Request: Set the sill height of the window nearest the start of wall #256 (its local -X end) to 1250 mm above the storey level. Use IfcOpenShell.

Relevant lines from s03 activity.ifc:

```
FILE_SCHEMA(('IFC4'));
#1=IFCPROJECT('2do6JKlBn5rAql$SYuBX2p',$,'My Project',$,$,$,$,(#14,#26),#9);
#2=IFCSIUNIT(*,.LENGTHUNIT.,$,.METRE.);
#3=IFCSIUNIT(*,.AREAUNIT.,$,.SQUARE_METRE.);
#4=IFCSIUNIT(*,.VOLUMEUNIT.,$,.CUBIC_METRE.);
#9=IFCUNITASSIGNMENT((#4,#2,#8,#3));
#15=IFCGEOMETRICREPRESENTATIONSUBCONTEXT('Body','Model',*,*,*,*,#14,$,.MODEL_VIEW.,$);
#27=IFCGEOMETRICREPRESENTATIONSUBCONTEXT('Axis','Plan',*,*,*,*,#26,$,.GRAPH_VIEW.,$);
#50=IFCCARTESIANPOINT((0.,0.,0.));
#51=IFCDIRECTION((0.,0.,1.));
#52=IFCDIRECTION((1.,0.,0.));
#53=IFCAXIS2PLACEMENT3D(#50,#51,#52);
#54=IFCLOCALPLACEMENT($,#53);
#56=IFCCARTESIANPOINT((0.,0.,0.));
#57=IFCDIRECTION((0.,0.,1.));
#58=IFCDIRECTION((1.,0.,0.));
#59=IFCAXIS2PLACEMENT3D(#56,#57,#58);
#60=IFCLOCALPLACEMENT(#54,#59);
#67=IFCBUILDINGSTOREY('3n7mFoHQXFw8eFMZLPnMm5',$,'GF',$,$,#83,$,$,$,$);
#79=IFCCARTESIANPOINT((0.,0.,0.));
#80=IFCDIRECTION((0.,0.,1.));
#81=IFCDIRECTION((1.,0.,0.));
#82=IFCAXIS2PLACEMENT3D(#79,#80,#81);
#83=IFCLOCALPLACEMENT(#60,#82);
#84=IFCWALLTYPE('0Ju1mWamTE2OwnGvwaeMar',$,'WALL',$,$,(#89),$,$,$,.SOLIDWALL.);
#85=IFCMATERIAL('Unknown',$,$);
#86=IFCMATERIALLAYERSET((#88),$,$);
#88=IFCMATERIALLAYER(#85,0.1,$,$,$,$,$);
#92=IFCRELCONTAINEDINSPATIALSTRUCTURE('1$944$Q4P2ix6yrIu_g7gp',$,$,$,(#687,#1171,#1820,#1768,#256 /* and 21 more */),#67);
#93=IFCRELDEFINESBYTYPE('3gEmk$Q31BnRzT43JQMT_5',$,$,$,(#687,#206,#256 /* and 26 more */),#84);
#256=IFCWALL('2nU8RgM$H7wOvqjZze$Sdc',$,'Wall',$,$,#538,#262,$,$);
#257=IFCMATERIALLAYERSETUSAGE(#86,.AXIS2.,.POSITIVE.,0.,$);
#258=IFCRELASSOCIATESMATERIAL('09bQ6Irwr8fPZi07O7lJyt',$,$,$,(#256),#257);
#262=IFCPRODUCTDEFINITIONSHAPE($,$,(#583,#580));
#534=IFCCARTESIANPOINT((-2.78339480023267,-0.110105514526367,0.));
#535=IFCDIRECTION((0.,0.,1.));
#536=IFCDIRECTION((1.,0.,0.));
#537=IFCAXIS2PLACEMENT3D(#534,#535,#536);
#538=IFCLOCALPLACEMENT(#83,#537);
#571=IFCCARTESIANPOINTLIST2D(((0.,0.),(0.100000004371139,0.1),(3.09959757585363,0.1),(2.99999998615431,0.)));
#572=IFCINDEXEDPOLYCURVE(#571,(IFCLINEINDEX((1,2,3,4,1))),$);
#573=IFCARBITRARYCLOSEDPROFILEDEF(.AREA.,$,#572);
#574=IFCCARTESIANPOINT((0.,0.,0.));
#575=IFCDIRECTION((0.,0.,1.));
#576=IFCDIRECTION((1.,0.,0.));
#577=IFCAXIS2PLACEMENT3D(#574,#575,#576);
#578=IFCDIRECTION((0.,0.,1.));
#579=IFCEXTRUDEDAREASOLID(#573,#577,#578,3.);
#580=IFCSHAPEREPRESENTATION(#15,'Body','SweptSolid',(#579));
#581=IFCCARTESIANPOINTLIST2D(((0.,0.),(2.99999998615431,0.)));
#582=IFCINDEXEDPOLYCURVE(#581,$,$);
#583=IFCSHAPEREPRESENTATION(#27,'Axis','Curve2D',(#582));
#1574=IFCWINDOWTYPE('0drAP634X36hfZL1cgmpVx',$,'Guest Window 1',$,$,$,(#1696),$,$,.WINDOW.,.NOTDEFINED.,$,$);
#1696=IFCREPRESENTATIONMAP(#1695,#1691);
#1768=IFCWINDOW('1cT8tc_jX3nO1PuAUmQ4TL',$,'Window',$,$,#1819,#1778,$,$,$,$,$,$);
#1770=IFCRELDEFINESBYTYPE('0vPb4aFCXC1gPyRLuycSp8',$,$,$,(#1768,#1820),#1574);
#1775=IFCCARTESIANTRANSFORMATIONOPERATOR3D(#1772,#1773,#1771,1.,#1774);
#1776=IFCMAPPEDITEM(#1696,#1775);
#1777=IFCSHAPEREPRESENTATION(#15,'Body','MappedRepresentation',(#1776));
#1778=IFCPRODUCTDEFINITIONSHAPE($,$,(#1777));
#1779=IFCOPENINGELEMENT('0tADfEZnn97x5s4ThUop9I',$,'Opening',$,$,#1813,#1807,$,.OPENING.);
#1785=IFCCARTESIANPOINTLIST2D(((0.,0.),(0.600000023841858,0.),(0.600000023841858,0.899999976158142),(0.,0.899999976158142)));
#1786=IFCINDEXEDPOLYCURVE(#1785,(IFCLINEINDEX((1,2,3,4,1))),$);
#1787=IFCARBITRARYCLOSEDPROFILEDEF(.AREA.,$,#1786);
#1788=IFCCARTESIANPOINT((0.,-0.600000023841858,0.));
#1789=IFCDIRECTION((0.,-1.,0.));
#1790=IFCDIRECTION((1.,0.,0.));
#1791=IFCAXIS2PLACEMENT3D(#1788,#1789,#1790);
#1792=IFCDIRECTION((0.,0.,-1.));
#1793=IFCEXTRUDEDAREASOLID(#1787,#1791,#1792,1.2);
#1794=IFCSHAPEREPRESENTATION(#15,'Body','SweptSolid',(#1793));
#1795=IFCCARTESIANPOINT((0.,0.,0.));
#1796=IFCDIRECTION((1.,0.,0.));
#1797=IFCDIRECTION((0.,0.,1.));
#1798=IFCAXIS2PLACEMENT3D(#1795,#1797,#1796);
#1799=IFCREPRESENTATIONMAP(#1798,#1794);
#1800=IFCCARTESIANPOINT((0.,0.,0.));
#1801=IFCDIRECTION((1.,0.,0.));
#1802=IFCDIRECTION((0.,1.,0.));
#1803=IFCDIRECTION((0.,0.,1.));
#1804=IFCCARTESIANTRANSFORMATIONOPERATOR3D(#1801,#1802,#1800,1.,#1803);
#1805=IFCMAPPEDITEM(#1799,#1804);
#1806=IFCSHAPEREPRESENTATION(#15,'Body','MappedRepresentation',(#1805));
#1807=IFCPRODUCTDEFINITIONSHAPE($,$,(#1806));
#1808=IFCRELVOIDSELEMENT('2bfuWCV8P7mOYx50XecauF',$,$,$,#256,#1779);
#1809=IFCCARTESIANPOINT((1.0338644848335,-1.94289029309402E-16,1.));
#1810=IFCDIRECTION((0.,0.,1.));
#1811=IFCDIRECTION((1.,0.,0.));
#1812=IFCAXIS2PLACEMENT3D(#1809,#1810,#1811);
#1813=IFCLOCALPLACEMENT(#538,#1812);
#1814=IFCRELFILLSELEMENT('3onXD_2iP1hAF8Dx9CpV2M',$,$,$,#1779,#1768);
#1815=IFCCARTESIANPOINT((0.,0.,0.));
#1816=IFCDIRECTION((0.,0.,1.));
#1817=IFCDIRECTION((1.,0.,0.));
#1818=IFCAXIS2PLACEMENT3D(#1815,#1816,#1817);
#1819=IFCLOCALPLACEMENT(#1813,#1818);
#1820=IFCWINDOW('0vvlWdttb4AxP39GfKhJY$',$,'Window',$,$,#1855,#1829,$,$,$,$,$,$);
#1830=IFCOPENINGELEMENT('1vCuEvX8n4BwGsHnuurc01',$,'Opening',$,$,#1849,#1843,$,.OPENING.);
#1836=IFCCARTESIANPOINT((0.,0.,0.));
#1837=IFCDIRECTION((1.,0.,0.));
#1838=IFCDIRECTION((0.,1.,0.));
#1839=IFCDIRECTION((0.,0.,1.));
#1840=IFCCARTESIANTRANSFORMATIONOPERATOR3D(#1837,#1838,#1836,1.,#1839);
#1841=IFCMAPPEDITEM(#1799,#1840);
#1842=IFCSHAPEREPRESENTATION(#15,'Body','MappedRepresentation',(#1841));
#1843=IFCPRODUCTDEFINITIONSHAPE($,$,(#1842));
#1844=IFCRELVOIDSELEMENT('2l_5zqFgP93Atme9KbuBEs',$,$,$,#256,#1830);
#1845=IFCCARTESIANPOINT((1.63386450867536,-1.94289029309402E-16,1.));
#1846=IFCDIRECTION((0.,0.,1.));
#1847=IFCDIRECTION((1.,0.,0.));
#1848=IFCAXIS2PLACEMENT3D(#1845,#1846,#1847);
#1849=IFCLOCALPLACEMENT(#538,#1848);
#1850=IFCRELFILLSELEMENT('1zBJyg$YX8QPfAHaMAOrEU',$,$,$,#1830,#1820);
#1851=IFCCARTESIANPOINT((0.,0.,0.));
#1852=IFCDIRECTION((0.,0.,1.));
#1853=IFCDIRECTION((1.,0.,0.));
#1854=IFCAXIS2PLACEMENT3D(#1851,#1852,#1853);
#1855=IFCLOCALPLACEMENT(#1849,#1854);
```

```python
import numpy as np
import ifcopenshell
import ifcopenshell.api.geometry
import ifcopenshell.geom
import ifcopenshell.util.element
import ifcopenshell.util.placement
import ifcopenshell.util.shape
import ifcopenshell.util.unit

model = ifcopenshell.open("s03 activity.ifc")
unit_scale = ifcopenshell.util.unit.calculate_unit_scale(model)

window = model.by_id(1768)
opening = window.FillsVoids[0].RelatingOpeningElement
storey = ifcopenshell.util.element.get_container(window, ifc_class="IfcBuildingStorey")
level = ifcopenshell.util.placement.get_local_placement(storey.ObjectPlacement)[2, 3]

# The opening's origin need not be at the sill, so measure its lowest point.
shape = ifcopenshell.geom.create_shape(ifcopenshell.geom.settings(), opening)
bottom = ifcopenshell.util.shape.get_shape_bottom_elevation(shape, shape.geometry) / unit_scale
dz = level + 1.25 / unit_scale - bottom

shift = np.array([0.0, 0.0, dz])
# The window is placed relative to its opening, so it follows when the opening moves.
matrix = ifcopenshell.util.placement.get_local_placement(opening.ObjectPlacement)
matrix[:3, 3] += shift
ifcopenshell.api.geometry.edit_object_placement(
    model, product=opening, matrix=matrix, is_si=False, should_transform_children=True
)

print(f"moved by {dz * unit_scale:+.3f} m")

model.write("s03 activity_edited.ifc")
```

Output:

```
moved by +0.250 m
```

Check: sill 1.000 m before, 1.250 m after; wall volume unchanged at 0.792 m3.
